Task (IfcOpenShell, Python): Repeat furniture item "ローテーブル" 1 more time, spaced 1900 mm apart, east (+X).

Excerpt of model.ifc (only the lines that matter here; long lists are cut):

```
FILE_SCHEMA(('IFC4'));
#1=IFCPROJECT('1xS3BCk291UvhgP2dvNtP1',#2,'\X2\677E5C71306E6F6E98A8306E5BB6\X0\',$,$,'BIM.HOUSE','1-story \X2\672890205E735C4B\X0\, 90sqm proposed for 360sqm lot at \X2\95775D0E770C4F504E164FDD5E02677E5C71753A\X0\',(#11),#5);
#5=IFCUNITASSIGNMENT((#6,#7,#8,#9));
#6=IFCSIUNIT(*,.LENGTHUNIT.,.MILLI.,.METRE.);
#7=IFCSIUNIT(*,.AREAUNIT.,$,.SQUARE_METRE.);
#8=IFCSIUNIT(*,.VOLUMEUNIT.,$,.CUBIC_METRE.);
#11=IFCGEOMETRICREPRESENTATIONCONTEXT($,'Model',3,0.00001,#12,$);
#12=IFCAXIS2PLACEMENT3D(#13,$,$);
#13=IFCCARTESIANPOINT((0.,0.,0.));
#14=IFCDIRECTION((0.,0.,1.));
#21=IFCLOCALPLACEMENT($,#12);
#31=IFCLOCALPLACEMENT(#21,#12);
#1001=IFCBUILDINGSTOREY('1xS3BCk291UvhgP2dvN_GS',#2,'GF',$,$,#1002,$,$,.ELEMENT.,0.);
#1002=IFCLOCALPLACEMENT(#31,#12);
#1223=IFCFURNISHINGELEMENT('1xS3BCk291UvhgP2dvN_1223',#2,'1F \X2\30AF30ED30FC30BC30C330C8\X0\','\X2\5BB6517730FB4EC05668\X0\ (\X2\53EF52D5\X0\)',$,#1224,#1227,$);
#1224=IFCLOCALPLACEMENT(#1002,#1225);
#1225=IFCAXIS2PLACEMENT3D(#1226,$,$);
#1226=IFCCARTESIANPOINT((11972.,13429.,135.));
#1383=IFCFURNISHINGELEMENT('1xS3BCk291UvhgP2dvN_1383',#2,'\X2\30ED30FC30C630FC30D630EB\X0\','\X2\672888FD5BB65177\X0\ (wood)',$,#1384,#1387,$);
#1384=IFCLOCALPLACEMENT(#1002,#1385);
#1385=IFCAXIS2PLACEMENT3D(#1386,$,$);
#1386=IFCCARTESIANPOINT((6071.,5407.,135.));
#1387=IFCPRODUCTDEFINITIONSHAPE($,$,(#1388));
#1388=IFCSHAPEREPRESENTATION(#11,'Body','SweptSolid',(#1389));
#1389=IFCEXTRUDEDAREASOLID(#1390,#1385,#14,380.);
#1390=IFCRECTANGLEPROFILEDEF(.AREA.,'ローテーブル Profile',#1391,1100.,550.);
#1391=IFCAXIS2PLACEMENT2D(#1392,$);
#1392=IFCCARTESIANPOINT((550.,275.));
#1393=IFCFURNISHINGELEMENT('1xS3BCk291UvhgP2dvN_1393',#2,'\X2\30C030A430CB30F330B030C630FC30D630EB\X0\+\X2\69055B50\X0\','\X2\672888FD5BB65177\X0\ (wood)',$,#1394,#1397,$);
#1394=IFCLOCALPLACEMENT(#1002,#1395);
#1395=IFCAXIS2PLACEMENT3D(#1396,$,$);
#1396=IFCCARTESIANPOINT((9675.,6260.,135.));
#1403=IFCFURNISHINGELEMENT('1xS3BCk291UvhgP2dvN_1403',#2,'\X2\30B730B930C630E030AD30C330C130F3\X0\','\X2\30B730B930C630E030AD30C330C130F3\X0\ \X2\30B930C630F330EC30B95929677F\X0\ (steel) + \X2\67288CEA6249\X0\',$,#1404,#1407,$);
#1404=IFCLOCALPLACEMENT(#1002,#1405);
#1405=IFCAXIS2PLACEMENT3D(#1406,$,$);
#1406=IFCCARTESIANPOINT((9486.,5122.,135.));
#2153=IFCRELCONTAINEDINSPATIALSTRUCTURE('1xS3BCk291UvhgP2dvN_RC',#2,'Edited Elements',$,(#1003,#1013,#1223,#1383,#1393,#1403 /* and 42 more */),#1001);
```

```python
import numpy as np
import ifcopenshell
import ifcopenshell.api.geometry
import ifcopenshell.api.root
import ifcopenshell.util.element
import ifcopenshell.util.placement
import ifcopenshell.util.unit

model = ifcopenshell.open("model.ifc")
unit_scale = ifcopenshell.util.unit.calculate_unit_scale(model)


def reuse_history(source, copy):
    """copy_class also copies each property set's owner history, people and application; keep the originals."""
    for rel in copy.IsDefinedBy:
        if rel.is_a("IfcRelDefinesByProperties") and (history := rel.RelatingPropertyDefinition.OwnerHistory):
            rel.RelatingPropertyDefinition.OwnerHistory = source.OwnerHistory
            ifcopenshell.util.element.remove_deep2(model, history)


source = model.by_id(1383)
base = ifcopenshell.util.placement.get_local_placement(source.ObjectPlacement)
step = np.array([1.0, 0.0, 0.0]) * 1.9 / unit_scale

for i in range(1, 2):
    copy = ifcopenshell.api.root.copy_class(model, product=source)
    copy.Representation = ifcopenshell.util.element.copy_deep(
        model, source.Representation, exclude=["IfcGeometricRepresentationContext", "IfcRepresentationMap"]
    )
    reuse_history(source, copy)
    matrix = base.copy()
    matrix[:3, 3] += i * step
    print("added at", matrix[:3, 3].round(3) + 0.0)
    ifcopenshell.api.geometry.edit_object_placement(model, product=copy, matrix=matrix, is_si=False)

model.write("model_v2.ifc")
```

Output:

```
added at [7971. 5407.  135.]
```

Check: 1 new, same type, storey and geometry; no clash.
